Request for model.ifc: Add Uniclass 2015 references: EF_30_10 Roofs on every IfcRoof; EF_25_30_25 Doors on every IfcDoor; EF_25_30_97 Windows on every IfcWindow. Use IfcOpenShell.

First a look at what the model holds.

```python
import ifcopenshell

model = ifcopenshell.open("model.ifc")
print(model.schema)
print("classifications:", [c.Name for c in model.by_type("IfcClassification")])
for ifc_class in ("IfcDoor", "IfcRoof", "IfcStair", "IfcWall", "IfcWindow"):
    print(ifc_class, len(model.by_type(ifc_class)))
```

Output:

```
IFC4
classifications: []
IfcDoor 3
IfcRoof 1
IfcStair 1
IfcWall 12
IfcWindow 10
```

```python
import ifcopenshell
import ifcopenshell.api.classification

model = ifcopenshell.open("model.ifc")

system = ifcopenshell.api.classification.add_classification(model, classification="Uniclass 2015")

codes = {
    "IfcRoof": ("EF_30_10", "Roofs"),
    "IfcDoor": ("EF_25_30_25", "Doors"),
    "IfcWindow": ("EF_25_30_97", "Windows"),
}
for ifc_class, (code, name) in codes.items():
    products = model.by_type(ifc_class)
    ifcopenshell.api.classification.add_reference(
        model, products=products, classification=system, identification=code, name=name
    )
    print(code, len(products))

model.write("model_rev.ifc")
```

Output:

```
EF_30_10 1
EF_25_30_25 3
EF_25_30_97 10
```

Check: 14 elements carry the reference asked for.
